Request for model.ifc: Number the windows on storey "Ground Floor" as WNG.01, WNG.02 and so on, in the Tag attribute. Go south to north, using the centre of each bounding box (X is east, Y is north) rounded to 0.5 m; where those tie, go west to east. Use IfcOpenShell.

First a look at what the model holds.

```python
import ifcopenshell
import ifcopenshell.util.element
import ifcopenshell.util.placement

model = ifcopenshell.open("model.ifc")
print(model.schema)
storey = next(s for s in model.by_type("IfcBuildingStorey") if s.Name == "Ground Floor")
windows = [e for e in ifcopenshell.util.element.get_decomposition(storey) if e.is_a("IfcWindow")]
for e in sorted(windows, key=lambda e: e.id()):
    origin = ifcopenshell.util.placement.get_local_placement(e.ObjectPlacement)[:3, 3]
    print(e.id(), e.Tag, e.Name, origin.round(2) + 0.0, sep=" | ")
```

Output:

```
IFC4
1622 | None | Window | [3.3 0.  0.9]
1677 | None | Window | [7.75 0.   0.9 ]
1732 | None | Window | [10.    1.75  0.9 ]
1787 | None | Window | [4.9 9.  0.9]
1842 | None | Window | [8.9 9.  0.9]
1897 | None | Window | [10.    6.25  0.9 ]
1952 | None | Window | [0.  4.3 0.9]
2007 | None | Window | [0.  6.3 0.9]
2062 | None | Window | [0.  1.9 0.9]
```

```python
import ifcopenshell
import ifcopenshell.geom
import ifcopenshell.util.element
import ifcopenshell.util.shape

model = ifcopenshell.open("model.ifc")
settings = ifcopenshell.geom.settings()
settings.set("use-world-coords", True)


def centre(element):
    shape = ifcopenshell.geom.create_shape(settings, element)
    return ifcopenshell.util.shape.get_bbox_centroid(shape.geometry)


storey = next(s for s in model.by_type("IfcBuildingStorey") if s.Name == "Ground Floor")
windows = [e for e in ifcopenshell.util.element.get_decomposition(storey) if e.is_a("IfcWindow")]

# Insertion points can sit at a corner or the storey origin, so sort by the geometry (in metres).
centres = {e: centre(e) for e in windows}
windows.sort(key=lambda e: (round(centres[e][1] / 0.5), centres[e][0]))

for i, e in enumerate(windows, start=1):
    number = f"WNG.{i:02d}"
    e.Tag = number
    print(e.id(), number)

model.write("model_updated.ifc")
```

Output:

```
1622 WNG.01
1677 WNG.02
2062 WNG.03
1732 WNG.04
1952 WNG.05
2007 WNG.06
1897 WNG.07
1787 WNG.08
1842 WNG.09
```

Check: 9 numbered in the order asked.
